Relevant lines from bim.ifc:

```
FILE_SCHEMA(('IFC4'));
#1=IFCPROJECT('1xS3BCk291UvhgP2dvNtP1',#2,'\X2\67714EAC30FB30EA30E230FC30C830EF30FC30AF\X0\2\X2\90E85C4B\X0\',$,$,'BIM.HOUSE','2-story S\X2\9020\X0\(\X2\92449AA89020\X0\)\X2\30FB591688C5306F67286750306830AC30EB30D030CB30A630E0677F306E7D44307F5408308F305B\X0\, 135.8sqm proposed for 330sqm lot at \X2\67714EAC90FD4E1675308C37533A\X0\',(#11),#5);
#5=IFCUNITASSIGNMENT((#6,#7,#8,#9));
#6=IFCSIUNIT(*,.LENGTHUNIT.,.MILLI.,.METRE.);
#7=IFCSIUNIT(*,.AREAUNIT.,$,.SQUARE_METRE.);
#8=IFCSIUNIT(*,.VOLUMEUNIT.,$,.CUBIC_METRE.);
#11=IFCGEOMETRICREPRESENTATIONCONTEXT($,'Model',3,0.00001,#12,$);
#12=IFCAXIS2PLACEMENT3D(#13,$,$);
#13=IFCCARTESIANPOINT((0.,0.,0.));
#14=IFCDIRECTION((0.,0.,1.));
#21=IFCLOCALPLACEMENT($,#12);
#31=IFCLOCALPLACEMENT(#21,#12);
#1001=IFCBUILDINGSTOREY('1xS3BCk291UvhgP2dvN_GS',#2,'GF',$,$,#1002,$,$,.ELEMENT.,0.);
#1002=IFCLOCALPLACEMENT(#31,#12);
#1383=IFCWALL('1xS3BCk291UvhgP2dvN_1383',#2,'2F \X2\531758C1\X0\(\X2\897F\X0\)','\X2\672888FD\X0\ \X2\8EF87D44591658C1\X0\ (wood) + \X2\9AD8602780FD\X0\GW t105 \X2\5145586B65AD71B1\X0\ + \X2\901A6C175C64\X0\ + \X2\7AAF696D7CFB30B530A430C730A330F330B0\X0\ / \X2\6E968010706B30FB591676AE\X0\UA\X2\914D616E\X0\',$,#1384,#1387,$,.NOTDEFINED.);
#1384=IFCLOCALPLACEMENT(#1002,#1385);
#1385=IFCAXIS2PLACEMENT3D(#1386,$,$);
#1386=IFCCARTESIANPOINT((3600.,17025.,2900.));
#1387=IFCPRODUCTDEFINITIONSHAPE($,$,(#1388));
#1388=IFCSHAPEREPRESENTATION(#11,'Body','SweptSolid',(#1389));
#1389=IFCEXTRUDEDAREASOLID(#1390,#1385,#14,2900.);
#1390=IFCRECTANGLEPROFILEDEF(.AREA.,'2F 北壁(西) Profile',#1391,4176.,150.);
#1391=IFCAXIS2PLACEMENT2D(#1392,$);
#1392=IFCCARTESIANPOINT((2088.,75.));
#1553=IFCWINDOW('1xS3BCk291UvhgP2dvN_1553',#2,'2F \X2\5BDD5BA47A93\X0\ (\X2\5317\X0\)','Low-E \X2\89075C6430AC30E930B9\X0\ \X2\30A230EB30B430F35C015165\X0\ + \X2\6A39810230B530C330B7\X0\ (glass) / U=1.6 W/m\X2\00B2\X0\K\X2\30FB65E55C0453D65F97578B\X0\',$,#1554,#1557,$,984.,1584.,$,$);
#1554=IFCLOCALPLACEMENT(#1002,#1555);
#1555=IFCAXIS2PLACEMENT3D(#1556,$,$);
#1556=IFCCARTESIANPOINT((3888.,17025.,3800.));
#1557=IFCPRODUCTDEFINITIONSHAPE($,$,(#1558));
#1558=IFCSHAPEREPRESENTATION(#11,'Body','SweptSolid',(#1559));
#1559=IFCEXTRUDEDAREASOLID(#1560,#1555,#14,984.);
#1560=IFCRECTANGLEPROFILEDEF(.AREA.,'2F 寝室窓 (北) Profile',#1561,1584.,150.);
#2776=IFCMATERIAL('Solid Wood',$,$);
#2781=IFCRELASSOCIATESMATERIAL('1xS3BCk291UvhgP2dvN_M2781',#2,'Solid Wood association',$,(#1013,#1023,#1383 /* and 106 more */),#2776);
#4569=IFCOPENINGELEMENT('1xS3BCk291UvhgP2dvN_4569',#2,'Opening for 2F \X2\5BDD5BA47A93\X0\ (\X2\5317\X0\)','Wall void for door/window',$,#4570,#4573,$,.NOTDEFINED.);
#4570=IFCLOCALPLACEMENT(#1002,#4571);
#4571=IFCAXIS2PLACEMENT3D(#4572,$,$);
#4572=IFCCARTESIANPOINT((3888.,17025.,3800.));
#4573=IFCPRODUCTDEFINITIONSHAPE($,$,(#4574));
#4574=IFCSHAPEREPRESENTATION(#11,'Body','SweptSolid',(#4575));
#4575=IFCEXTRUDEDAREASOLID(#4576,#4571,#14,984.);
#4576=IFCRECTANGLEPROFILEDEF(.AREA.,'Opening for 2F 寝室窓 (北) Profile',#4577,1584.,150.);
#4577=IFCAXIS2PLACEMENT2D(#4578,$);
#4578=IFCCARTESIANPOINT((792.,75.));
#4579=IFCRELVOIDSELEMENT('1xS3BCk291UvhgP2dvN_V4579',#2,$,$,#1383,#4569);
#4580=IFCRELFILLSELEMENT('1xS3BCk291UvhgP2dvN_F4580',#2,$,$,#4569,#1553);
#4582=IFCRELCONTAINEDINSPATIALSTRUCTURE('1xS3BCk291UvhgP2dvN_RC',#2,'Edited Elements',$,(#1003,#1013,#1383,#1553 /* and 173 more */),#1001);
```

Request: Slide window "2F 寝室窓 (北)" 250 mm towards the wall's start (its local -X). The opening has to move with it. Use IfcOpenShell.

```python
import ifcopenshell
import ifcopenshell.api.geometry
import ifcopenshell.util.placement
import ifcopenshell.util.unit

model = ifcopenshell.open("bim.ifc")
unit_scale = ifcopenshell.util.unit.calculate_unit_scale(model)

window = model.by_guid("1xS3BCk291UvhgP2dvN_1553")
opening = window.FillsVoids[0].RelatingOpeningElement
wall = opening.VoidsElements[0].RelatingBuildingElement

wall_matrix = ifcopenshell.util.placement.get_local_placement(wall.ObjectPlacement)
shift = wall_matrix[:3, 0] * -0.25 / unit_scale
before = ifcopenshell.util.placement.get_local_placement(window.ObjectPlacement)[:3, 3].copy()

# The window is not placed relative to its opening, so move both.
for product in (opening, window):
    matrix = ifcopenshell.util.placement.get_local_placement(product.ObjectPlacement)
    matrix[:3, 3] += shift
    ifcopenshell.api.geometry.edit_object_placement(model, product=product, matrix=matrix, is_si=False)

after = ifcopenshell.util.placement.get_local_placement(window.ObjectPlacement)[:3, 3]
print("window moved by", (after - before).round(3) + 0.0)

model.write("bim_updated.ifc")
```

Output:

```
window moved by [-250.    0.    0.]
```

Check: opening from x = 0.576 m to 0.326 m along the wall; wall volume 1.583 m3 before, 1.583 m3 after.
